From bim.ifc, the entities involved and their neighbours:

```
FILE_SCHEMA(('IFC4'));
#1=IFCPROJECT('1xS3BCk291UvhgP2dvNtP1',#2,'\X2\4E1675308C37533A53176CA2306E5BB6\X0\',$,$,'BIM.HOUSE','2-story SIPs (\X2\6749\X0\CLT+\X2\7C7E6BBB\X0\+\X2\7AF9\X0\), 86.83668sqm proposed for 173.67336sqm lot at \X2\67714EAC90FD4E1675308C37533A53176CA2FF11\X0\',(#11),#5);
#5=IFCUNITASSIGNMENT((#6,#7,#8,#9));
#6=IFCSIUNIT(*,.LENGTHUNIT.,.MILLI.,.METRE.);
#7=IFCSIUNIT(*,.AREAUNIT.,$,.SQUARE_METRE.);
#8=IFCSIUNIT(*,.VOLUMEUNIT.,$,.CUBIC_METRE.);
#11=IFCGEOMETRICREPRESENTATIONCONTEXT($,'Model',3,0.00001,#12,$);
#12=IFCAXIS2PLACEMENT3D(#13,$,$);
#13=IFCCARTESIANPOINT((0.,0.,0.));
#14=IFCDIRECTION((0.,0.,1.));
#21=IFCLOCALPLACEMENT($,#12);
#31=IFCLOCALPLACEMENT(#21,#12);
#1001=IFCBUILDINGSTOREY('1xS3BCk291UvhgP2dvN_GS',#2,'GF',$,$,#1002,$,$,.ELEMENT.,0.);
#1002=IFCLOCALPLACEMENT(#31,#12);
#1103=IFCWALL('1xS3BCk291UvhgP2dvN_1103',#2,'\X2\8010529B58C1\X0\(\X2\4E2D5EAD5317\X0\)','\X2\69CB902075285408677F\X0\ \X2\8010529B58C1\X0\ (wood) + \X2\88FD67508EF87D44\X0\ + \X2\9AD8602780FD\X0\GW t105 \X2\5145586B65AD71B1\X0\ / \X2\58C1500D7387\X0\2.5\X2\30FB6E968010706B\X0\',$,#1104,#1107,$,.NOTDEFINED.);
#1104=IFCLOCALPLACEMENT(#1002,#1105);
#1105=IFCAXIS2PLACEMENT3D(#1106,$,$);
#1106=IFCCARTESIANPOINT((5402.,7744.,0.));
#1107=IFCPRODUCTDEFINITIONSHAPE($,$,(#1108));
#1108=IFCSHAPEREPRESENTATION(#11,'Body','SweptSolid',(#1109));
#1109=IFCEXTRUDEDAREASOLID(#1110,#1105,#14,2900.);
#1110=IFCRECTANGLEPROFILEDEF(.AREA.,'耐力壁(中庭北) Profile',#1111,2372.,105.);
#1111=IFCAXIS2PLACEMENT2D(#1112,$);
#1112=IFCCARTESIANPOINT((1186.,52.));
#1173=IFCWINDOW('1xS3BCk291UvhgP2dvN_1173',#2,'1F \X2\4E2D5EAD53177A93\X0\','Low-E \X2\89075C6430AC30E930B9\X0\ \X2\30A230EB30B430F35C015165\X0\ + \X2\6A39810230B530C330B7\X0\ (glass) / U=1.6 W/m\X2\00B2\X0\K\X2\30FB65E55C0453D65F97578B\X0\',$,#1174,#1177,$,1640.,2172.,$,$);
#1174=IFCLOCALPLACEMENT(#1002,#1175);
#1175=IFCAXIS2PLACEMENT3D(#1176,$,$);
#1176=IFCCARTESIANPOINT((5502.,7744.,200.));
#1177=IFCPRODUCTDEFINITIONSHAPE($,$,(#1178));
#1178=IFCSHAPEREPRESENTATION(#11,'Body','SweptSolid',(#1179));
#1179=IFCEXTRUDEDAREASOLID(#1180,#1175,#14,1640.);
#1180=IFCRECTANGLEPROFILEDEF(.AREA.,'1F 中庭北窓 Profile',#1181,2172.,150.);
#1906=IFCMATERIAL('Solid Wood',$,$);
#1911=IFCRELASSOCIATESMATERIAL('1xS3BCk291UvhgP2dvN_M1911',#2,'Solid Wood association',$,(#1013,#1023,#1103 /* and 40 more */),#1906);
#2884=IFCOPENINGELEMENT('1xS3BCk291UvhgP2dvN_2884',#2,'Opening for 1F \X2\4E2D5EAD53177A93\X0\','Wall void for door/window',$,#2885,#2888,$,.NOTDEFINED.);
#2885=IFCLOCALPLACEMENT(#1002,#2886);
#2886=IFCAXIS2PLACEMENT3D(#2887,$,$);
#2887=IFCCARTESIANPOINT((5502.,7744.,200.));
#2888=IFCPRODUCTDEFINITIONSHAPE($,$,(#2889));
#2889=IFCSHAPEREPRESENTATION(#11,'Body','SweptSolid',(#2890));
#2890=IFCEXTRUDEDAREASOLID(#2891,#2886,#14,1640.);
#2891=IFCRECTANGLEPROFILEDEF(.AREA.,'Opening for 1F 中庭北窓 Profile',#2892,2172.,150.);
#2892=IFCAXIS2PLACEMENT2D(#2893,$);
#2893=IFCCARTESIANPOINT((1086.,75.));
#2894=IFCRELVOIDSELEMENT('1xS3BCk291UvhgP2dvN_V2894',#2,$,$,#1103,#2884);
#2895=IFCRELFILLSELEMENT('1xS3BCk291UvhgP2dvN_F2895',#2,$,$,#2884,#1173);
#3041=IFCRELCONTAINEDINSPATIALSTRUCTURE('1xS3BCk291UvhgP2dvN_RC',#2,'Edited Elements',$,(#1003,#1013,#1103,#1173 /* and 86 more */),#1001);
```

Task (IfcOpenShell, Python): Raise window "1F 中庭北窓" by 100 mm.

```python
import numpy as np
import ifcopenshell
import ifcopenshell.api.geometry
import ifcopenshell.util.placement
import ifcopenshell.util.unit

model = ifcopenshell.open("bim.ifc")
unit_scale = ifcopenshell.util.unit.calculate_unit_scale(model)

window = model.by_guid("1xS3BCk291UvhgP2dvN_1173")
opening = window.FillsVoids[0].RelatingOpeningElement
dz = 0.1 / unit_scale

shift = np.array([0.0, 0.0, dz])
# The window is not placed relative to its opening, so move both.
for product in (opening, window):
    matrix = ifcopenshell.util.placement.get_local_placement(product.ObjectPlacement)
    matrix[:3, 3] += shift
    ifcopenshell.api.geometry.edit_object_placement(model, product=product, matrix=matrix, is_si=False)

print(f"moved by {dz * unit_scale:+.3f} m")

model.write("bim_updated.ifc")
```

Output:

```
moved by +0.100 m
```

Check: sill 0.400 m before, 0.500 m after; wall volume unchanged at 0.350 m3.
